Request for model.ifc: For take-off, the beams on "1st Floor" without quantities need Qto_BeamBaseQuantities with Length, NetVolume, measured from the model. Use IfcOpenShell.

First a look at what the model holds.

```python
import ifcopenshell
import ifcopenshell.util.element
import ifcopenshell.util.unit

model = ifcopenshell.open("model.ifc")
print(model.schema)
for unit_type in ("LENGTHUNIT", "AREAUNIT", "VOLUMEUNIT"):
    print(unit_type, ifcopenshell.util.unit.calculate_unit_scale(model, unit_type))
storey = next(s for s in model.by_type("IfcBuildingStorey") if s.Name == "1st Floor")
beams = [e for e in ifcopenshell.util.element.get_decomposition(storey) if e.is_a("IfcBeam")]
for e in sorted(beams, key=lambda e: e.id()):
    print(e.id(), e.is_a(), e.Name, list(ifcopenshell.util.element.get_psets(e, qtos_only=True)), sep=" | ")
```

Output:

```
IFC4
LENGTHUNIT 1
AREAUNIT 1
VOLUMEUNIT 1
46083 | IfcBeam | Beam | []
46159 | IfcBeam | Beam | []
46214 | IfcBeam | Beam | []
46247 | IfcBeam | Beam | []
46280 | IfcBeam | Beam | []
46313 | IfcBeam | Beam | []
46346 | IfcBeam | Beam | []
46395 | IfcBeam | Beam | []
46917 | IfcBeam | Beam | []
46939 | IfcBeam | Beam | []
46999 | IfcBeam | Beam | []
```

```python
import ifcopenshell
import ifcopenshell.api.pset
import ifcopenshell.geom
import ifcopenshell.util.element
import ifcopenshell.util.shape
import ifcopenshell.util.unit

model = ifcopenshell.open("model.ifc")
unit_scale = ifcopenshell.util.unit.calculate_unit_scale(model)
volume_scale = ifcopenshell.util.unit.calculate_unit_scale(model, "VOLUMEUNIT")
settings = ifcopenshell.geom.settings()

storey = next(s for s in model.by_type("IfcBuildingStorey") if s.Name == "1st Floor")
beams = [e for e in ifcopenshell.util.element.get_decomposition(storey) if e.is_a("IfcBeam")]

for e in sorted(beams, key=lambda e: e.id()):
    if ifcopenshell.util.element.get_psets(e, qtos_only=True, should_inherit=False):
        continue
    # Geometry comes back in metres, in the element's own axes.
    shape = ifcopenshell.geom.create_shape(settings, e)
    values = {
        "Length": ifcopenshell.util.shape.get_max_xyz(shape.geometry) / unit_scale,
        "NetVolume": ifcopenshell.util.shape.get_volume(shape.geometry) / volume_scale,
    }
    qto = ifcopenshell.api.pset.add_qto(model, product=e, name="Qto_BeamBaseQuantities")
    ifcopenshell.api.pset.edit_qto(model, qto=qto, properties=values)
    print(e.id(), {k: round(v, 3) for k, v in values.items()})

model.write("model_v2.ifc")
```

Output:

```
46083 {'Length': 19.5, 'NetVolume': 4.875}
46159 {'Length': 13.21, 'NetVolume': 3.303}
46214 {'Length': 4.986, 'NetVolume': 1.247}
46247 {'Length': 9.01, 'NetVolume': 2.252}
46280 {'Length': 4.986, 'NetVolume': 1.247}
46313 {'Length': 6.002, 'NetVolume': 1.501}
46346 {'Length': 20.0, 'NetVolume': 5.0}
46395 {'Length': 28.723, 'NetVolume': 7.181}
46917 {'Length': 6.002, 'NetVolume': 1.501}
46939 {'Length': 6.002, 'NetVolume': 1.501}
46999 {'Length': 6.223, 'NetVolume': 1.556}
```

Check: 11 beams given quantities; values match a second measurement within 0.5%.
